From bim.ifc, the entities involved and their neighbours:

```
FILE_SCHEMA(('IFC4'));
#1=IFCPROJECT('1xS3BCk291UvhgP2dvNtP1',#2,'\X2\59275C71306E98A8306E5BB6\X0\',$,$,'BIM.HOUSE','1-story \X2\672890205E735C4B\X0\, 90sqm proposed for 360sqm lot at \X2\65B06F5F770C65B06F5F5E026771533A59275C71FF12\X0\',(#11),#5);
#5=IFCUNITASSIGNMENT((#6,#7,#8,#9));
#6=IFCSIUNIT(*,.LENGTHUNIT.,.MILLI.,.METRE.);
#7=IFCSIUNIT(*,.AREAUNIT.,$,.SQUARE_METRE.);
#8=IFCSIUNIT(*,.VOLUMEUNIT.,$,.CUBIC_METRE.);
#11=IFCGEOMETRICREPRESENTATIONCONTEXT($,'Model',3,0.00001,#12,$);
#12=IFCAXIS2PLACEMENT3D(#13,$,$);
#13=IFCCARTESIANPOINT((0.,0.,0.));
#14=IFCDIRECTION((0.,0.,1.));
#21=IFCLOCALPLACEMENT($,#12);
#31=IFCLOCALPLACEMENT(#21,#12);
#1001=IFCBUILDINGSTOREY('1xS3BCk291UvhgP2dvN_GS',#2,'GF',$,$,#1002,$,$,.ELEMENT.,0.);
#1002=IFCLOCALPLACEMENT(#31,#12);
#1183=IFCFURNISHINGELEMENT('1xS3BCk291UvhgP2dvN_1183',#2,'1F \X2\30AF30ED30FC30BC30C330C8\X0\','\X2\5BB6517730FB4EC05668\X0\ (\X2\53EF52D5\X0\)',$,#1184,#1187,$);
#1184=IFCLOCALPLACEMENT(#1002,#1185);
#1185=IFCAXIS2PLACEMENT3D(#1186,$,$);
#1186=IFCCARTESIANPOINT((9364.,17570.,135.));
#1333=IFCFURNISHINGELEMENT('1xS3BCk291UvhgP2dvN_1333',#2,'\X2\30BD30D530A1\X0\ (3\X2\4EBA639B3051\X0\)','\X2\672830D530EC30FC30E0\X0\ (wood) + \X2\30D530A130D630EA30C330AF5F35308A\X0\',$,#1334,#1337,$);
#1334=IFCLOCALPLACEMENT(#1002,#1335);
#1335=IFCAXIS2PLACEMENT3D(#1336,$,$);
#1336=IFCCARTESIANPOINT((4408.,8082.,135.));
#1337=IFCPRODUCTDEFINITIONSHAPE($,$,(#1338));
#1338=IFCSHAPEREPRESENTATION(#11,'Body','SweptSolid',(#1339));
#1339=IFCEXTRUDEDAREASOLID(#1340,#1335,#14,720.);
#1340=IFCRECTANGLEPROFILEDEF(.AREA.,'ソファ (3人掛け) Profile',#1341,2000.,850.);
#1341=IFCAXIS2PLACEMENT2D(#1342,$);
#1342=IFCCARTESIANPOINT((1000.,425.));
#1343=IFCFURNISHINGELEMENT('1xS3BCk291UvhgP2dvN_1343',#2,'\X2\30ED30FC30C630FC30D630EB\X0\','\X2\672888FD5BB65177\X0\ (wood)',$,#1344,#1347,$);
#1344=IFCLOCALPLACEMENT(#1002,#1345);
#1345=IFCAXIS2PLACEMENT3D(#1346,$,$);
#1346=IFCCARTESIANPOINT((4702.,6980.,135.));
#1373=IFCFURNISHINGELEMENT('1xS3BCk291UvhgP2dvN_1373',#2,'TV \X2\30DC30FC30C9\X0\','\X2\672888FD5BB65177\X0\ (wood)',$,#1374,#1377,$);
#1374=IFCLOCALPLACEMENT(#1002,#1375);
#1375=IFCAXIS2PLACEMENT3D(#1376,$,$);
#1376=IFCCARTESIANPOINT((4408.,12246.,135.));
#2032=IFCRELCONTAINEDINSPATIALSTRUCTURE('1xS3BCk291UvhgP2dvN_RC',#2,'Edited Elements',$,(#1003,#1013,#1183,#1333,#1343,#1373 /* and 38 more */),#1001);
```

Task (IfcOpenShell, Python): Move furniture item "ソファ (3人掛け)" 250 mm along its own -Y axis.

```python
import ifcopenshell
import ifcopenshell.api.geometry
import ifcopenshell.util.placement

model = ifcopenshell.open("bim.ifc")

item = model.by_guid("1xS3BCk291UvhgP2dvN_1333")
matrix = ifcopenshell.util.placement.get_local_placement(item.ObjectPlacement)
matrix[:3, 3] -= matrix[:3, 1] * 250.0
ifcopenshell.api.geometry.edit_object_placement(model, product=item, matrix=matrix, is_si=False)

print(ifcopenshell.util.placement.get_local_placement(item.ObjectPlacement).round(3) + 0.0)

model.write("bim_v2.ifc")
```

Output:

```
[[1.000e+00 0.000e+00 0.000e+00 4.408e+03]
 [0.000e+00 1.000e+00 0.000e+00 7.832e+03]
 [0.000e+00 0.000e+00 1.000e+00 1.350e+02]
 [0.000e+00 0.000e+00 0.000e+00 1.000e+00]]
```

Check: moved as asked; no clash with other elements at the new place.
